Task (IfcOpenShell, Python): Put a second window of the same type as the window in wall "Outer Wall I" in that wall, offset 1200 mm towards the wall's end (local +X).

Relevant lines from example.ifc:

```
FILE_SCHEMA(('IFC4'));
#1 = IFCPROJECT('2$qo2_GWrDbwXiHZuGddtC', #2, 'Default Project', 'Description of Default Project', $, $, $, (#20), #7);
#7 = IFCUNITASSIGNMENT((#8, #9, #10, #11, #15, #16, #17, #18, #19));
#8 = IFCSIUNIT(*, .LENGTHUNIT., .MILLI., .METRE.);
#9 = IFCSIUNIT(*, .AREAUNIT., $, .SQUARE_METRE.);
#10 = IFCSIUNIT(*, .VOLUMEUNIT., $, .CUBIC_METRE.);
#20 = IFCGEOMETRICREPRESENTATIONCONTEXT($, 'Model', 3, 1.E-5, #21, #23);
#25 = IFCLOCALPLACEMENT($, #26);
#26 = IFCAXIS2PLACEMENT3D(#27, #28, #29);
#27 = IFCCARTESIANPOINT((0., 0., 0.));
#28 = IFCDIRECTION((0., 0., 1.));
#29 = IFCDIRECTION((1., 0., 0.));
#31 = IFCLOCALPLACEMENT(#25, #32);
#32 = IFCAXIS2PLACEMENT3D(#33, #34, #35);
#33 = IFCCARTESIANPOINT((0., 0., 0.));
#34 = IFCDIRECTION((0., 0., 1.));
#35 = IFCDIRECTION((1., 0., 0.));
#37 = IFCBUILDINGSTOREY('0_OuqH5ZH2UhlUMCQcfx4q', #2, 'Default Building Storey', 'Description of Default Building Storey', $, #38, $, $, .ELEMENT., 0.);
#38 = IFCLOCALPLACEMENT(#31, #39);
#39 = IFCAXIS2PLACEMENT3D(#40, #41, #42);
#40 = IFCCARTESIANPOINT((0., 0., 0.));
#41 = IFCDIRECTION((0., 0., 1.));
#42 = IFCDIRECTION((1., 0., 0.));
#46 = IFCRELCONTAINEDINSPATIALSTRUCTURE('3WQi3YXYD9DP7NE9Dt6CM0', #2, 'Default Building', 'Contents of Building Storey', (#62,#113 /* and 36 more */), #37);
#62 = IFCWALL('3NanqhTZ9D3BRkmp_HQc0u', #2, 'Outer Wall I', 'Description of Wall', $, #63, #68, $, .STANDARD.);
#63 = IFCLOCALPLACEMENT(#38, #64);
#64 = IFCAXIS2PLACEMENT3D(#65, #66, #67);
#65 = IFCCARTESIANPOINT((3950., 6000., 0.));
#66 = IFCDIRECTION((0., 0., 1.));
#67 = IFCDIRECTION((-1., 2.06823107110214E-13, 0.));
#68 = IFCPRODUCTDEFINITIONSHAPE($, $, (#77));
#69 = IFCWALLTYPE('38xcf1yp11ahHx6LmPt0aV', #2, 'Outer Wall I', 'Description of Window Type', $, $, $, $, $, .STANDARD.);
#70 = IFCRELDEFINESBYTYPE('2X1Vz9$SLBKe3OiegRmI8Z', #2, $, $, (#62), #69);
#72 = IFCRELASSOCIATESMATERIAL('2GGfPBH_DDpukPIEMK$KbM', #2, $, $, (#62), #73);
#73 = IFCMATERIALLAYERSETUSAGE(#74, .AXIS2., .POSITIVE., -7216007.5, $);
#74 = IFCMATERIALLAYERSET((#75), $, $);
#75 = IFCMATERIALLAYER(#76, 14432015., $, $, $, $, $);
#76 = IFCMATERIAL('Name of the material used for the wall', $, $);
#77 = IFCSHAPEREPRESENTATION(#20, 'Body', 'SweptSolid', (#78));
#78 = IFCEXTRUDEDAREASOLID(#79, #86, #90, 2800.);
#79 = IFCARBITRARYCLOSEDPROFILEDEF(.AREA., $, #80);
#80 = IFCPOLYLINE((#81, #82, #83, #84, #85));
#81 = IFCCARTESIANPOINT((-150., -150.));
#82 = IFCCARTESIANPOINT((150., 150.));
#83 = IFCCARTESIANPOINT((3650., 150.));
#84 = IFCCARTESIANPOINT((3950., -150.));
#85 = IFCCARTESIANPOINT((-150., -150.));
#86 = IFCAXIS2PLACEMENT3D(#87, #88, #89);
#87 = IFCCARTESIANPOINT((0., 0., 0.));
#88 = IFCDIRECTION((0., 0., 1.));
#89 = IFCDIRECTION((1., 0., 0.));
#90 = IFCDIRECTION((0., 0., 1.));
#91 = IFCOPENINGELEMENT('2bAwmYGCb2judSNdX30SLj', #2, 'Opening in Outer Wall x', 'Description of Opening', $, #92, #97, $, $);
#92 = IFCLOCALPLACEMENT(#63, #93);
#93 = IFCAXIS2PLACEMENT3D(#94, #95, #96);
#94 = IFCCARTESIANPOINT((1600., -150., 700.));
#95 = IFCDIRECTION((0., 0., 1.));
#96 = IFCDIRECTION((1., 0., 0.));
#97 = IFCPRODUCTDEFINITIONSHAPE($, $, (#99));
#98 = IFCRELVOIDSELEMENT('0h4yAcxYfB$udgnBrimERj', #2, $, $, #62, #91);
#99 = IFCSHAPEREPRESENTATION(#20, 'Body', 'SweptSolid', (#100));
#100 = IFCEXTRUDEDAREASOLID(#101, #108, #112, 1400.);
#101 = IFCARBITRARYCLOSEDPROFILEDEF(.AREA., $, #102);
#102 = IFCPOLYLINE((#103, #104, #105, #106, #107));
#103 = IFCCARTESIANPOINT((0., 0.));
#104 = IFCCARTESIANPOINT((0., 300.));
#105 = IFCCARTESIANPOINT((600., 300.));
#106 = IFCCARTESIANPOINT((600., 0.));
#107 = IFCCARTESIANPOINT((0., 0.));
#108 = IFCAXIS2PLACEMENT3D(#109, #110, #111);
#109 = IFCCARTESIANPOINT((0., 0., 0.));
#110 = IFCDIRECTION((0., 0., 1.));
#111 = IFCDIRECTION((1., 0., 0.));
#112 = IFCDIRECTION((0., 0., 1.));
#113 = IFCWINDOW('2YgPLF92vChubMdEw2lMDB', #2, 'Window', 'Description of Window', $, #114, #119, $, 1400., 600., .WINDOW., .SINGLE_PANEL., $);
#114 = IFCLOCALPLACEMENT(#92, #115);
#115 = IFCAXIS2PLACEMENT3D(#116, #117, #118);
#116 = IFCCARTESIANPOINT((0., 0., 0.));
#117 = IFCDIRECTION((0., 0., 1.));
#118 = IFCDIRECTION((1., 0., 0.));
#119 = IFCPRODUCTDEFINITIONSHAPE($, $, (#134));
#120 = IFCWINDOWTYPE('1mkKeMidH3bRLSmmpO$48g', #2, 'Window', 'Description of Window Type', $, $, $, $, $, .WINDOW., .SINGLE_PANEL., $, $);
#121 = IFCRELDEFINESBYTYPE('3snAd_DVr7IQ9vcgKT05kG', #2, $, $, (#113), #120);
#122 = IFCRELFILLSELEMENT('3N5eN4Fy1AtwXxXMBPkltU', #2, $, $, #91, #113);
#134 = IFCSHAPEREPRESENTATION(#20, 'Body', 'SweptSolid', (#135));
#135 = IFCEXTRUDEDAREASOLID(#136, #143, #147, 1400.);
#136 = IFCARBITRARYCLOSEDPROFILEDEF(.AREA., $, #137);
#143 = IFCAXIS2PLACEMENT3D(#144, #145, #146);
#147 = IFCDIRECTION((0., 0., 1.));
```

```python
import ifcopenshell
import ifcopenshell.api.feature
import ifcopenshell.api.geometry
import ifcopenshell.api.root
import ifcopenshell.geom
import ifcopenshell.util.element
import ifcopenshell.util.placement
import ifcopenshell.util.shape
import ifcopenshell.util.unit

model = ifcopenshell.open("example.ifc")
unit_scale = ifcopenshell.util.unit.calculate_unit_scale(model)
settings = ifcopenshell.geom.settings()


def volume(element):
    """Net volume in cubic metres, openings subtracted."""
    shape = ifcopenshell.geom.create_shape(settings, element)
    return ifcopenshell.util.shape.get_volume(shape.geometry)


def reuse_history(source, copy):
    """copy_class also copies each property set's owner history, people and application; keep the originals."""
    for rel in copy.IsDefinedBy:
        if rel.is_a("IfcRelDefinesByProperties") and (history := rel.RelatingPropertyDefinition.OwnerHistory):
            rel.RelatingPropertyDefinition.OwnerHistory = source.OwnerHistory
            ifcopenshell.util.element.remove_deep2(model, history)


window = model.by_guid("2YgPLF92vChubMdEw2lMDB")
opening = window.FillsVoids[0].RelatingOpeningElement
wall = opening.VoidsElements[0].RelatingBuildingElement
before = volume(wall)
shift = ifcopenshell.util.placement.get_local_placement(wall.ObjectPlacement)[:3, 0] * 1.2 / unit_scale

# copy_class copies the void relationship, type, container and properties, but no geometry.
new_opening = ifcopenshell.api.root.copy_class(model, product=opening)
new_opening.Representation = ifcopenshell.util.element.copy_deep(
    model, opening.Representation, exclude=["IfcGeometricRepresentationContext", "IfcRepresentationMap"]
)
new_window = ifcopenshell.api.root.copy_class(model, product=window)
new_window.Representation = ifcopenshell.util.element.copy_deep(
    model, window.Representation, exclude=["IfcGeometricRepresentationContext", "IfcRepresentationMap"]
)
reuse_history(window, new_window)
ifcopenshell.api.feature.add_filling(model, opening=new_opening, element=new_window)

for old, new in ((opening, new_opening), (window, new_window)):
    matrix = ifcopenshell.util.placement.get_local_placement(old.ObjectPlacement)
    matrix[:3, 3] += shift
    ifcopenshell.api.geometry.edit_object_placement(model, product=new, matrix=matrix, is_si=False)

after = volume(wall)

print(f"wall volume {before:.3f} -> {after:.3f} m3")

model.write("example_edited.ifc")
```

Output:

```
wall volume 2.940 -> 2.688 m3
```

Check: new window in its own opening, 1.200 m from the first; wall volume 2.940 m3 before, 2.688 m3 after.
